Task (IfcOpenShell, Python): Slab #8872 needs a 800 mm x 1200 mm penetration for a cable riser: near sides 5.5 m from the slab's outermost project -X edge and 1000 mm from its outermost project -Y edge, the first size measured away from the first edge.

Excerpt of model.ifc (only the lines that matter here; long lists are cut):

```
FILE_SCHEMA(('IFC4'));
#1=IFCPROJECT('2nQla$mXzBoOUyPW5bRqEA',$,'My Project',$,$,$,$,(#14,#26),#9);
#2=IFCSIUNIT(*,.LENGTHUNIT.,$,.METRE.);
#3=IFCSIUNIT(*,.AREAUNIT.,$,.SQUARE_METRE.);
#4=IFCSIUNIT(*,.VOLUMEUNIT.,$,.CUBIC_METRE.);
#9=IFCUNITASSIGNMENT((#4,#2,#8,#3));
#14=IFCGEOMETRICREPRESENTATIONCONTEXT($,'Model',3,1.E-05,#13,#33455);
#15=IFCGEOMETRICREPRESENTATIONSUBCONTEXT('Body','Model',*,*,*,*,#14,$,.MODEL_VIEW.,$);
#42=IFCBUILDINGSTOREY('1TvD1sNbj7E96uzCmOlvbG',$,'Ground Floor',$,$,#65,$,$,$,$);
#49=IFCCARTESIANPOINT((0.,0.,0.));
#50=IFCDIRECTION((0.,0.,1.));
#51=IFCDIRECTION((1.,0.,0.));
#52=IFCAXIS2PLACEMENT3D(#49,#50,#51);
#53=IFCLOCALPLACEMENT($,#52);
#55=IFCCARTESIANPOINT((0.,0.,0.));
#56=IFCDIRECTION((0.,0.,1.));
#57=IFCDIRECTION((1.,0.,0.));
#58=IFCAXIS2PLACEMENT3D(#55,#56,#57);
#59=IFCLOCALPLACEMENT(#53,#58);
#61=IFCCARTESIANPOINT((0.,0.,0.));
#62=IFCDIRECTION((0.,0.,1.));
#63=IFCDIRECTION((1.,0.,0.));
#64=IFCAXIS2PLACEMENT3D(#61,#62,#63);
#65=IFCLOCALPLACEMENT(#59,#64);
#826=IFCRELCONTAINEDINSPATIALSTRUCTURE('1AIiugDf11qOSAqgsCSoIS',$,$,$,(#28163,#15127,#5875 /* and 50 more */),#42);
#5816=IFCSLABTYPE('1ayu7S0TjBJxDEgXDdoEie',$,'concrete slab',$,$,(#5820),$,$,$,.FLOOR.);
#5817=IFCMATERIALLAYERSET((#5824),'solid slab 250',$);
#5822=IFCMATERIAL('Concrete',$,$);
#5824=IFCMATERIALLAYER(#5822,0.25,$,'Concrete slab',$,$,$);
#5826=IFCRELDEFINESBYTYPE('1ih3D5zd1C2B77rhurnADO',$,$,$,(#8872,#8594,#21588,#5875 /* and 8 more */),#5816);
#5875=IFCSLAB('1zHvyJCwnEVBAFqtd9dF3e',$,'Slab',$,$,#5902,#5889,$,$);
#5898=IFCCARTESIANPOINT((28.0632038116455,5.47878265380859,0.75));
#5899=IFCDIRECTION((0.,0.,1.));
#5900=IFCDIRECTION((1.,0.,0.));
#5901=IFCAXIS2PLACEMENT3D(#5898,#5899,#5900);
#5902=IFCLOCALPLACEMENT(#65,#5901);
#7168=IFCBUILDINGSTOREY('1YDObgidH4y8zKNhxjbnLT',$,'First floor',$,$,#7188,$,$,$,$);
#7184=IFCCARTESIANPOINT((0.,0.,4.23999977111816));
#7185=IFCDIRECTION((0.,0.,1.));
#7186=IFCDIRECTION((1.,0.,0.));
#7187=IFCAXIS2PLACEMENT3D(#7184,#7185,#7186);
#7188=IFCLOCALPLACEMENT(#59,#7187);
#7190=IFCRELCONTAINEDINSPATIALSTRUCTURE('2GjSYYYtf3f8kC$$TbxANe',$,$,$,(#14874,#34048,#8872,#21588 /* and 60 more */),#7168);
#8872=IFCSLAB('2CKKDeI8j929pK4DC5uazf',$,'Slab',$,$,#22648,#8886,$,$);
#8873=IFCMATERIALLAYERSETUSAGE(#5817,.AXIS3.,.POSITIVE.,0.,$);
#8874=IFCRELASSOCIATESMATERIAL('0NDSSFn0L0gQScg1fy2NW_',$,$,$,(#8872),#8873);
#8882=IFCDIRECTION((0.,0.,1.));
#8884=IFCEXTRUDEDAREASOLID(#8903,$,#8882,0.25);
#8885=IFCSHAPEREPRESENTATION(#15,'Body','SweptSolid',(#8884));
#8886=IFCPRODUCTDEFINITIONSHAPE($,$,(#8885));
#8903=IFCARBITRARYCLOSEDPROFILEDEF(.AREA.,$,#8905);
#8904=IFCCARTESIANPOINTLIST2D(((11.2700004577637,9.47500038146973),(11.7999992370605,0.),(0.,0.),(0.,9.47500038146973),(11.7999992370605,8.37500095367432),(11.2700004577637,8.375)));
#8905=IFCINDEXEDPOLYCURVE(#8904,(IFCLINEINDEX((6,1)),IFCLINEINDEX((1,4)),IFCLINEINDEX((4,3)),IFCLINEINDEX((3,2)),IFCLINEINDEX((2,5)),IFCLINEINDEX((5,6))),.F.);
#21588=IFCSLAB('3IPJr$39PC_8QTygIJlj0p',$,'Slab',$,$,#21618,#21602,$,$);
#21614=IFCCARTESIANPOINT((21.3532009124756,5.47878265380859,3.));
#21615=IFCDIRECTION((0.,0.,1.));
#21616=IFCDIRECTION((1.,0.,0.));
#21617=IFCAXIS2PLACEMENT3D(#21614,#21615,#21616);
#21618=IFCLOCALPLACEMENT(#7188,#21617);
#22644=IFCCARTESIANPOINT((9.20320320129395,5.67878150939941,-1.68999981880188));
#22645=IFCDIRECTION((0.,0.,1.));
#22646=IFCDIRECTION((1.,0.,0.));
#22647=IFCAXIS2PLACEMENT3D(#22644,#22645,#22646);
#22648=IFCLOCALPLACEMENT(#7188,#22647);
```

```python
import numpy as np
import ifcopenshell
import ifcopenshell.api.feature
import ifcopenshell.api.geometry
import ifcopenshell.api.root
import ifcopenshell.geom
import ifcopenshell.util.placement
import ifcopenshell.util.representation
import ifcopenshell.util.shape
import ifcopenshell.util.unit

model = ifcopenshell.open("model.ifc")
unit_scale = ifcopenshell.util.unit.calculate_unit_scale(model)
settings = ifcopenshell.geom.settings()


def volume(element):
    """Net volume in cubic metres, openings subtracted."""
    shape = ifcopenshell.geom.create_shape(settings, element)
    return ifcopenshell.util.shape.get_volume(shape.geometry)


slab = model.by_guid("2CKKDeI8j929pK4DC5uazf")
before = volume(slab)

# Extent in the slab's own axes, in metres. The edges named are its -X and -Y sides.
slab_shape = ifcopenshell.geom.create_shape(settings, slab)
vertices = ifcopenshell.util.shape.get_vertices(slab_shape.geometry)
x_min, y_min, bottom = vertices.min(axis=0)
top = vertices[:, 2].max()

opening = ifcopenshell.api.root.create_entity(model, ifc_class="IfcOpeningElement", name="Cable riser opening", predefined_type="OPENING")
context = ifcopenshell.util.representation.get_context(model, "Model", "Body", "MODEL_VIEW")
width, depth = 0.8, 1.2
outline = [(0.0, 0.0), (width, 0.0), (width, depth), (0.0, depth), (0.0, 0.0)]
# Overshoot both faces by 50 mm so the cut is clean.
shape = ifcopenshell.api.geometry.add_slab_representation(
    model, context=context, depth=top - bottom + 0.1, polyline=outline
)
ifcopenshell.api.geometry.assign_representation(model, product=opening, representation=shape)

matrix = ifcopenshell.util.placement.get_local_placement(slab.ObjectPlacement)
matrix[:, 3] = matrix @ np.append(np.array([x_min + 5.5, y_min + 1, bottom - 0.05]) / unit_scale, 1.0)
ifcopenshell.api.geometry.edit_object_placement(model, product=opening, matrix=matrix, is_si=False)
ifcopenshell.api.feature.add_feature(model, feature=opening, element=slab)

after = volume(slab)

print(f"slab volume {before:.3f} -> {after:.3f} m3")

model.write("model-out.ifc")
```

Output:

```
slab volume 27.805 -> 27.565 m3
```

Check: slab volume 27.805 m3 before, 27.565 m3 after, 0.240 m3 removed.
